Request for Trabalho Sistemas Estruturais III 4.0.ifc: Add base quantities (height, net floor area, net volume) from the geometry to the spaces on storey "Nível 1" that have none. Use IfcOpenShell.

First a look at what the model holds.

```python
import ifcopenshell
import ifcopenshell.util.element
import ifcopenshell.util.unit

model = ifcopenshell.open("Trabalho Sistemas Estruturais III 4.0.ifc")
print(model.schema)
for unit_type in ("LENGTHUNIT", "AREAUNIT", "VOLUMEUNIT"):
    print(unit_type, ifcopenshell.util.unit.calculate_unit_scale(model, unit_type))
storey = next(s for s in model.by_type("IfcBuildingStorey") if s.Name == "Nível 1")
spaces = [e for e in ifcopenshell.util.element.get_decomposition(storey) if e.is_a("IfcSpace")]
for e in sorted(spaces, key=lambda e: e.id()):
    print(e.id(), e.is_a(), e.Name, list(ifcopenshell.util.element.get_psets(e, qtos_only=True)), sep=" | ")
```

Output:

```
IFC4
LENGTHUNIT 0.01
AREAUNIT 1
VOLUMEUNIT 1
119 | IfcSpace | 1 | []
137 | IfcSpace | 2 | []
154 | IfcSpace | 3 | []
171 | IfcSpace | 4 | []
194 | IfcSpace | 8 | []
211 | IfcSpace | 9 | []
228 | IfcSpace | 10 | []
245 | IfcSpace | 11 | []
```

```python
import ifcopenshell
import ifcopenshell.api.pset
import ifcopenshell.geom
import ifcopenshell.util.element
import ifcopenshell.util.shape
import ifcopenshell.util.unit

model = ifcopenshell.open("Trabalho Sistemas Estruturais III 4.0.ifc")
unit_scale = ifcopenshell.util.unit.calculate_unit_scale(model)
area_scale = ifcopenshell.util.unit.calculate_unit_scale(model, "AREAUNIT")
volume_scale = ifcopenshell.util.unit.calculate_unit_scale(model, "VOLUMEUNIT")
settings = ifcopenshell.geom.settings()

storey = next(s for s in model.by_type("IfcBuildingStorey") if s.Name == "Nível 1")
spaces = [e for e in ifcopenshell.util.element.get_decomposition(storey) if e.is_a("IfcSpace")]

for e in sorted(spaces, key=lambda e: e.id()):
    if ifcopenshell.util.element.get_psets(e, qtos_only=True, should_inherit=False):
        continue
    # Geometry comes back in metres, in the element's own axes.
    shape = ifcopenshell.geom.create_shape(settings, e)
    values = {
        "Height": ifcopenshell.util.shape.get_z(shape.geometry) / unit_scale,
        "NetFloorArea": ifcopenshell.util.shape.get_footprint_area(shape.geometry) / area_scale,
        "NetVolume": ifcopenshell.util.shape.get_volume(shape.geometry) / volume_scale,
    }
    qto = ifcopenshell.api.pset.add_qto(model, product=e, name="Qto_SpaceBaseQuantities")
    ifcopenshell.api.pset.edit_qto(model, qto=qto, properties=values)
    print(e.id(), {k: round(v, 3) for k, v in values.items()})

model.write("Trabalho Sistemas Estruturais III 4.0-out.ifc")
```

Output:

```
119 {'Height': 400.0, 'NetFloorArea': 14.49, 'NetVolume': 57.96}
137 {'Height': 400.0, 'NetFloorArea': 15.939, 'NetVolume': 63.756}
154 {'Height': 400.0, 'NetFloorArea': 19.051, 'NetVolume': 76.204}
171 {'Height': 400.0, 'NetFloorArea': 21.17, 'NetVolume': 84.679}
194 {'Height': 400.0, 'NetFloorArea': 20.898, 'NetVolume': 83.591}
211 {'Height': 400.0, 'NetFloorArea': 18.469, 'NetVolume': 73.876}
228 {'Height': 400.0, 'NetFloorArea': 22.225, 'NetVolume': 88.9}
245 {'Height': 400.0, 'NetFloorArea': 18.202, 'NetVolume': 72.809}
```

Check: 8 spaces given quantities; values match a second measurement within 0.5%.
